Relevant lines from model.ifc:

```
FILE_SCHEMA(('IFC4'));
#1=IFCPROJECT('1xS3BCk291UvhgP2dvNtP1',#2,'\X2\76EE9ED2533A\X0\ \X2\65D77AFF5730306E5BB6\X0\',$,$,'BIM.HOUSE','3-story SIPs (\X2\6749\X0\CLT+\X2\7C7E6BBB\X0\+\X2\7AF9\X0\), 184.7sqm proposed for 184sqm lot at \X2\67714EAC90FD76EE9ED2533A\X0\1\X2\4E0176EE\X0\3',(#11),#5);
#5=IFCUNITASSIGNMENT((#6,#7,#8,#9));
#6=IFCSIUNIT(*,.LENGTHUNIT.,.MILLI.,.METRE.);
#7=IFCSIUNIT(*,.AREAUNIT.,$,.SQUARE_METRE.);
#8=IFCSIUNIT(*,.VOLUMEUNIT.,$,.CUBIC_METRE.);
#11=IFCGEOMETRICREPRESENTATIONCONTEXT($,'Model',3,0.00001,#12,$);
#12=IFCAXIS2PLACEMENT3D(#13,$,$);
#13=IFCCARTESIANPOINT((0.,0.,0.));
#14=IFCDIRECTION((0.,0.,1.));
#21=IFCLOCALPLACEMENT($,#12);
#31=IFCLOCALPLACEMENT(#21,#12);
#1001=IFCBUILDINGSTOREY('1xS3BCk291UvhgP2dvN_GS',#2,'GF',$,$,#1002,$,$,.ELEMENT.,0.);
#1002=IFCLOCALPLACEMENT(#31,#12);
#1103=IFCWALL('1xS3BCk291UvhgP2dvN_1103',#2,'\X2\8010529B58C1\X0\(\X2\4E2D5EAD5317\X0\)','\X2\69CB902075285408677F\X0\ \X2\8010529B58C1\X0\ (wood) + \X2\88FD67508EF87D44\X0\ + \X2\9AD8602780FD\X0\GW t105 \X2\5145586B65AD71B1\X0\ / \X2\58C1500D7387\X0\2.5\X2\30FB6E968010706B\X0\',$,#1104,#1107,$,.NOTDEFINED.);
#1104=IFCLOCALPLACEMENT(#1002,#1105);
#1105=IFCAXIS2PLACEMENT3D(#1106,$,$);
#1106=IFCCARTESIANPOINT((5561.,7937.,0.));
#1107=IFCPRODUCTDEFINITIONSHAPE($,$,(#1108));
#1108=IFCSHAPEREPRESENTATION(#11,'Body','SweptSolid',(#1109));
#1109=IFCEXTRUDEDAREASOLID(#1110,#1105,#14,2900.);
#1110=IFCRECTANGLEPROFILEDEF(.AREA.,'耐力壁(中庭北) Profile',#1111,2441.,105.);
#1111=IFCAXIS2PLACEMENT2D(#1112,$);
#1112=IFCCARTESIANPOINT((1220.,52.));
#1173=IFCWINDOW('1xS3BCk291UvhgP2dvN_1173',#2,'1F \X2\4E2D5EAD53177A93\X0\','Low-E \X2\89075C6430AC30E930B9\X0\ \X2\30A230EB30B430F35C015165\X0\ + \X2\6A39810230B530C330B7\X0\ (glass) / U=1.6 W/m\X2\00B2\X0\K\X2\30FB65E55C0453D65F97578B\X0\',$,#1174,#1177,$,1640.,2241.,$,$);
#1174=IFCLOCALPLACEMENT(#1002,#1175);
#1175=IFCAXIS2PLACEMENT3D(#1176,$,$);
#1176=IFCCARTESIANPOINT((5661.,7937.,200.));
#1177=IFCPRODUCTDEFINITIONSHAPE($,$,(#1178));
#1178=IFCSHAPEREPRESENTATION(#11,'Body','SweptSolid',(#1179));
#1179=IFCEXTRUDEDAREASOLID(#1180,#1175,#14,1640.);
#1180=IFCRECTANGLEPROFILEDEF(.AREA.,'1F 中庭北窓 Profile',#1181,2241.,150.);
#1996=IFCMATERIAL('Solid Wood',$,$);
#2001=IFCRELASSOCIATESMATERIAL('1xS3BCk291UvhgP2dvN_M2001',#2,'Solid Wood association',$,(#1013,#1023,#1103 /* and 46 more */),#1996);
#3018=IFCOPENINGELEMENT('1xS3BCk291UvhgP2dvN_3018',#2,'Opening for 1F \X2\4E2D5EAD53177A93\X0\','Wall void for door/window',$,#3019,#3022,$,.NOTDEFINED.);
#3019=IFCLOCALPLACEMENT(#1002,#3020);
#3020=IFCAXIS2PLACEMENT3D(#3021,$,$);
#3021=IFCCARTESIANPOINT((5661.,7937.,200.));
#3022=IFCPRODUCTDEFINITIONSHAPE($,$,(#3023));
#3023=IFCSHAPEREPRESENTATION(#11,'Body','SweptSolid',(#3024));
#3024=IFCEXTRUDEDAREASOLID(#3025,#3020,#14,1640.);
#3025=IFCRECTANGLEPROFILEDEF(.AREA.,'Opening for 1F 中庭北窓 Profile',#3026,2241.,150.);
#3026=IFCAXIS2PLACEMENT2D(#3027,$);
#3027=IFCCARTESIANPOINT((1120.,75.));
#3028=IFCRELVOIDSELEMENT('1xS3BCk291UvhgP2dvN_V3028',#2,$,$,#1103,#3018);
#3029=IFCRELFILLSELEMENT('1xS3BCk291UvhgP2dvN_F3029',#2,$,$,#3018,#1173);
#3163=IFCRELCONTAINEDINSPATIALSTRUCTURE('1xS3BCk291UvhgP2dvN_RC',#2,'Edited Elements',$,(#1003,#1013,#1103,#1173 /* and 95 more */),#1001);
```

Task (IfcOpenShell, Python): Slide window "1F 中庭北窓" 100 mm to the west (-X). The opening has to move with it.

```python
import ifcopenshell
import ifcopenshell.api.geometry
import ifcopenshell.util.placement

model = ifcopenshell.open("model.ifc")

window = model.by_guid("1xS3BCk291UvhgP2dvN_1173")
opening = window.FillsVoids[0].RelatingOpeningElement
wall = opening.VoidsElements[0].RelatingBuildingElement

wall_matrix = ifcopenshell.util.placement.get_local_placement(wall.ObjectPlacement)
shift = wall_matrix[:3, 0] * -100.0
before = ifcopenshell.util.placement.get_local_placement(window.ObjectPlacement)[:3, 3].copy()

# The window is not placed relative to its opening, so move both.
for product in (opening, window):
    matrix = ifcopenshell.util.placement.get_local_placement(product.ObjectPlacement)
    matrix[:3, 3] += shift
    ifcopenshell.api.geometry.edit_object_placement(model, product=product, matrix=matrix, is_si=False)

after = ifcopenshell.util.placement.get_local_placement(window.ObjectPlacement)[:3, 3]
print("window moved by", (after - before).round(3) + 0.0)

model.write("model_updated.ifc")
```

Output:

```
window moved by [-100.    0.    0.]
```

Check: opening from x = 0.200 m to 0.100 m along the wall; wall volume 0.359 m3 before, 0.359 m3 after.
